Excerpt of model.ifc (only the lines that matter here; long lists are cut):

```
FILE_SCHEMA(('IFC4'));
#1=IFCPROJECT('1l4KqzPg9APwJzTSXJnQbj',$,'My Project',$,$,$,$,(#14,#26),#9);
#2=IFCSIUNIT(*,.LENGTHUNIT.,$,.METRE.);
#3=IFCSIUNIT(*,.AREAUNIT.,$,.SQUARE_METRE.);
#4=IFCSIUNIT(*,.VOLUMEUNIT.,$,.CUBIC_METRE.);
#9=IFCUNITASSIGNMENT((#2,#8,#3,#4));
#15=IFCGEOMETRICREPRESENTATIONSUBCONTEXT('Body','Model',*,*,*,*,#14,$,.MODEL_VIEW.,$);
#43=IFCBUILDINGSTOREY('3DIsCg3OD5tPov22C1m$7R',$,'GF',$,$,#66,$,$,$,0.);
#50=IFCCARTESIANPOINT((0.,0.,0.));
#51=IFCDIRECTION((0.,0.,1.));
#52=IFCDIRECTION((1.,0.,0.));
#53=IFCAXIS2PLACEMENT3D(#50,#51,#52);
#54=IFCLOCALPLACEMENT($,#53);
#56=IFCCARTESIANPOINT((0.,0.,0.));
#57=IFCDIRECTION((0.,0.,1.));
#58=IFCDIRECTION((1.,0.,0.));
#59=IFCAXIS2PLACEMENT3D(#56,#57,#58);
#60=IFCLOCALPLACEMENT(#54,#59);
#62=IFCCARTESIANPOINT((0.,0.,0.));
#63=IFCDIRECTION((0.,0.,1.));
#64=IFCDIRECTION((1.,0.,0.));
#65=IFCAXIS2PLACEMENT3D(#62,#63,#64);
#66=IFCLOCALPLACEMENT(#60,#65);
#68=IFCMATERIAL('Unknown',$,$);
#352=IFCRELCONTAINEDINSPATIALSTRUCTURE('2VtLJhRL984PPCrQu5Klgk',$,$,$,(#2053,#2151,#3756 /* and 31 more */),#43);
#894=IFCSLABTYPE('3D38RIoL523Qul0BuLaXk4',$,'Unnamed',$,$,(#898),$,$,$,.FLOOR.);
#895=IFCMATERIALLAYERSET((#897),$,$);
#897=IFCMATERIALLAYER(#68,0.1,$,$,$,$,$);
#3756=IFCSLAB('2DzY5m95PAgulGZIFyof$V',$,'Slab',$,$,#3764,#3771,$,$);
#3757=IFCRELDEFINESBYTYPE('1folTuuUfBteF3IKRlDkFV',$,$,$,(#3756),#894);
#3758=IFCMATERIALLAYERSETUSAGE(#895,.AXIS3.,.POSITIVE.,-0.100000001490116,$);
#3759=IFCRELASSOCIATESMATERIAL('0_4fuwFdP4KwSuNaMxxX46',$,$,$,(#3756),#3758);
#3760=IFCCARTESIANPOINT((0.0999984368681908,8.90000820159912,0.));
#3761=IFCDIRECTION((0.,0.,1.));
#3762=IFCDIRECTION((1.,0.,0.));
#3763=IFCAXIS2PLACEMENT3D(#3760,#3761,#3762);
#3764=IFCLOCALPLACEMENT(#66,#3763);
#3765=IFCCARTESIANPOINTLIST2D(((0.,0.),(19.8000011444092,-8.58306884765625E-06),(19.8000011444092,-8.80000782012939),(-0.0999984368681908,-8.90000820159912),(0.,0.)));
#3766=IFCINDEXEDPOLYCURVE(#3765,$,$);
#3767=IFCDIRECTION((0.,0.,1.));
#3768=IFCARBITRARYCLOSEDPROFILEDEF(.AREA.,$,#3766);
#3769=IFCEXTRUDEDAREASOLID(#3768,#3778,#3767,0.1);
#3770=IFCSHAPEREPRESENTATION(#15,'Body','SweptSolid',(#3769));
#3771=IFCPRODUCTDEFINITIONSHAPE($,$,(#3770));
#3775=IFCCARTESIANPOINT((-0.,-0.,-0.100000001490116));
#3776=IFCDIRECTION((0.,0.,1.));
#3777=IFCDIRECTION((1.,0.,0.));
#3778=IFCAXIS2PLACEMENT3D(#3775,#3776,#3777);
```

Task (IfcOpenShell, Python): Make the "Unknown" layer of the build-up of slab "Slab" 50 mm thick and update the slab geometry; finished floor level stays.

```python
import ifcopenshell
import ifcopenshell.util.element
import ifcopenshell.util.representation
import ifcopenshell.util.unit

model = ifcopenshell.open("model.ifc")
unit_scale = ifcopenshell.util.unit.calculate_unit_scale(model)

layer_set = model.by_id(895)
layer = next(l for l in layer_set.MaterialLayers if l.Material and l.Material.Name == "Unknown")
change = 0.05 / unit_scale - layer.LayerThickness
layer.LayerThickness += change

# Geometry does not follow the layer set by itself.
slabs = [e for e in ifcopenshell.util.element.get_elements_by_material(model, layer_set) if e.is_a("IfcSlab")]
for slab in sorted(slabs, key=lambda e: e.id()):
    body = ifcopenshell.util.representation.get_representation(slab, "Model", "Body")
    solid = body.Items[0]
    old_depth = solid.Depth
    solid.Depth += change
    # Extruded upwards: lower the start of the extrusion so the top stays.
    x, y, z = solid.Position.Location.Coordinates
    solid.Position.Location = model.createIfcCartesianPoint((x, y, z - change))
    print(slab.id(), f"{old_depth:g} -> {solid.Depth:g}")

# The layers are counted up from the underside, which has moved.
for usage in {ifcopenshell.util.element.get_material(slab) for slab in slabs}:
    usage.OffsetFromReferenceLine -= change

model.write("model-out.ifc")
```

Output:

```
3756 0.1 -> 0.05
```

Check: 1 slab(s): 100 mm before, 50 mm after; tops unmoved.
